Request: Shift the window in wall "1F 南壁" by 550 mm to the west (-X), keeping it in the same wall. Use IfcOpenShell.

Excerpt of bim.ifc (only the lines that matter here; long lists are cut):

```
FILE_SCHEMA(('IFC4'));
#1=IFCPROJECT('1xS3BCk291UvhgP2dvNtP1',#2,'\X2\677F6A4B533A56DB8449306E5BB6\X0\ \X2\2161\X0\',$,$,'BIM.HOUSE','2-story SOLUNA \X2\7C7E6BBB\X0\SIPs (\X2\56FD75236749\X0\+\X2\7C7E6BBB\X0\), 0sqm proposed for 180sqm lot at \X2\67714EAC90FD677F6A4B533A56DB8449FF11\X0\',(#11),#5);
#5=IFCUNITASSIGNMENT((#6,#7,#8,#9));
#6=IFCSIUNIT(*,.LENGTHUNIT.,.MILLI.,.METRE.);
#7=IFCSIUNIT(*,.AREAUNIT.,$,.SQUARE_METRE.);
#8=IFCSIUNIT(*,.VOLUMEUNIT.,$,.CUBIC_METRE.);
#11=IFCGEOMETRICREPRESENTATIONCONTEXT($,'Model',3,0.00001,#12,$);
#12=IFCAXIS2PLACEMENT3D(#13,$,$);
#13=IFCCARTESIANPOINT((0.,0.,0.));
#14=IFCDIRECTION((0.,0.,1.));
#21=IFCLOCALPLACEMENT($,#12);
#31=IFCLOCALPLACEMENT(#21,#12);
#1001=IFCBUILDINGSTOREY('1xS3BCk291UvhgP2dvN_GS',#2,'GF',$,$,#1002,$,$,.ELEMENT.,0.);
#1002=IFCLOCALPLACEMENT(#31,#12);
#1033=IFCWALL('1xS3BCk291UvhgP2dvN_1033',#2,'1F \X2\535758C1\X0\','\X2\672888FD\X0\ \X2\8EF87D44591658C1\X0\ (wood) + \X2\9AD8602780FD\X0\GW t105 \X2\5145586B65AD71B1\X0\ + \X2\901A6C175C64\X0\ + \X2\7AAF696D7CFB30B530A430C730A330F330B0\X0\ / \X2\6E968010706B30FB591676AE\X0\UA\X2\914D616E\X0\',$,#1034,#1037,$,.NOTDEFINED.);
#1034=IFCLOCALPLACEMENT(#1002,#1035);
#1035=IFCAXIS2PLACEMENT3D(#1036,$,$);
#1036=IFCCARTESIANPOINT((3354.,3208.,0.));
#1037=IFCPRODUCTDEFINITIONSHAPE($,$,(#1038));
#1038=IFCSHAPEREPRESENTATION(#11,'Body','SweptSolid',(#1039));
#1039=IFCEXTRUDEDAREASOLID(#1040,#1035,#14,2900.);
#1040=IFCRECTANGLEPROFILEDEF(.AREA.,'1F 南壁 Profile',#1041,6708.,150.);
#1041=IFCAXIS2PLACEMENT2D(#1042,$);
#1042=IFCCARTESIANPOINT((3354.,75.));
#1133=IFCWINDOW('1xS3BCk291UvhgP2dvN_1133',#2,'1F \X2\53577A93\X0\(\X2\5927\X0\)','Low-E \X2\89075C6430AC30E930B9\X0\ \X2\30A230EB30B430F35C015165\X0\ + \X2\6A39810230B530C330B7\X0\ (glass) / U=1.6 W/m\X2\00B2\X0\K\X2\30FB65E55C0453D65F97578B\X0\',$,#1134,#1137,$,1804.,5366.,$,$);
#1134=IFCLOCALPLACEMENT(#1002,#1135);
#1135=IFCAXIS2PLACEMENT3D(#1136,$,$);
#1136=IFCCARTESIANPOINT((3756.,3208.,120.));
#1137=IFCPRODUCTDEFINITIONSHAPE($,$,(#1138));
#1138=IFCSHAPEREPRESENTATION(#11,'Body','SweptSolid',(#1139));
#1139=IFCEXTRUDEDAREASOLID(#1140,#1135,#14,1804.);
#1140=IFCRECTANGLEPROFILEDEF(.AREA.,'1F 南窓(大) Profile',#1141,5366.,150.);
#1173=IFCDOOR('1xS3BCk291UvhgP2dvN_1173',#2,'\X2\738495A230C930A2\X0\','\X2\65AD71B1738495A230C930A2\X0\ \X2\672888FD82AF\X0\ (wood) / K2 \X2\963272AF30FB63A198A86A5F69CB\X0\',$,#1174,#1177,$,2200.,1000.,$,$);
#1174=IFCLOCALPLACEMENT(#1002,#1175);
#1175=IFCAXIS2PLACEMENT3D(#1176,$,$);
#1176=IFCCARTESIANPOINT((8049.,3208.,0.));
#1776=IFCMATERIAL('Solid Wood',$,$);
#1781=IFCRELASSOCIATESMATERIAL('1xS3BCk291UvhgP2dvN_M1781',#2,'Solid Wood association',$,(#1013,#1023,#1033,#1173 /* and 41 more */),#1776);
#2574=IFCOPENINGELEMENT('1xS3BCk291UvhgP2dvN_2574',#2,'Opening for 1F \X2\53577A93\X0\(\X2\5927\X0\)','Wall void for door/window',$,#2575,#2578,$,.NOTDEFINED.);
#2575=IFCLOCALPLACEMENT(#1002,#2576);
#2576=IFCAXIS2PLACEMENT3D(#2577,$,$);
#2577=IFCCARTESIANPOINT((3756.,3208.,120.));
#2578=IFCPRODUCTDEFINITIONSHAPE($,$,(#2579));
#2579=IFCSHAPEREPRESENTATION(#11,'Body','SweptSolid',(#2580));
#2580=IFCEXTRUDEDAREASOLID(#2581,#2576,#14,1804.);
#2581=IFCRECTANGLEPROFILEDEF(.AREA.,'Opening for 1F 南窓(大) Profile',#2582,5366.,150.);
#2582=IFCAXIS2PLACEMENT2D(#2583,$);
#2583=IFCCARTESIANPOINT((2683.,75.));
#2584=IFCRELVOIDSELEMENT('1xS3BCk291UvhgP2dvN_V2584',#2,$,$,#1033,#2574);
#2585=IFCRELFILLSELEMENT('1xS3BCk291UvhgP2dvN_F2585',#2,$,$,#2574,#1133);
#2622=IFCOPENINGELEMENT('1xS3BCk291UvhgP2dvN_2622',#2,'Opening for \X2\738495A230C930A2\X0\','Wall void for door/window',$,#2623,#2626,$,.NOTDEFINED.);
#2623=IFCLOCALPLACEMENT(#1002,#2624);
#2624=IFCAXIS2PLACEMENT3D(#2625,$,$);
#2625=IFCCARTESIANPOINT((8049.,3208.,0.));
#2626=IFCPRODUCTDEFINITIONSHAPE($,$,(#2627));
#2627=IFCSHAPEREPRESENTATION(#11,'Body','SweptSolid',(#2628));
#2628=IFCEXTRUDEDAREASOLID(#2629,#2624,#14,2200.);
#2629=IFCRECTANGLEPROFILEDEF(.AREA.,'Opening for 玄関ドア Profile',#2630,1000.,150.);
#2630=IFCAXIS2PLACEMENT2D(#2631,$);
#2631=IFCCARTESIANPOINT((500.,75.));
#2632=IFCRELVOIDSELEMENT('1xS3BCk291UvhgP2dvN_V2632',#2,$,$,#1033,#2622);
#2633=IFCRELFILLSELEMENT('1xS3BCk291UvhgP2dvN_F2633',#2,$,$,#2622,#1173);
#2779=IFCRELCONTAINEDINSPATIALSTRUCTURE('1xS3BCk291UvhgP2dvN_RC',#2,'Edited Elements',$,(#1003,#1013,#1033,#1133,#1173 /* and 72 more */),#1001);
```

```python
import ifcopenshell
import ifcopenshell.api.geometry
import ifcopenshell.util.placement

model = ifcopenshell.open("bim.ifc")

window = model.by_guid("1xS3BCk291UvhgP2dvN_1133")
opening = window.FillsVoids[0].RelatingOpeningElement
wall = opening.VoidsElements[0].RelatingBuildingElement

wall_matrix = ifcopenshell.util.placement.get_local_placement(wall.ObjectPlacement)
shift = wall_matrix[:3, 0] * -550.0
before = ifcopenshell.util.placement.get_local_placement(window.ObjectPlacement)[:3, 3].copy()

# The window is not placed relative to its opening, so move both.
for product in (opening, window):
    matrix = ifcopenshell.util.placement.get_local_placement(product.ObjectPlacement)
    matrix[:3, 3] += shift
    ifcopenshell.api.geometry.edit_object_placement(model, product=product, matrix=matrix, is_si=False)

after = ifcopenshell.util.placement.get_local_placement(window.ObjectPlacement)[:3, 3]
print("window moved by", (after - before).round(3) + 0.0)

model.write("bim_v2.ifc")
```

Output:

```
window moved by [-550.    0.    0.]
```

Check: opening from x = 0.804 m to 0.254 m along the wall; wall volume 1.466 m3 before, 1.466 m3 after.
